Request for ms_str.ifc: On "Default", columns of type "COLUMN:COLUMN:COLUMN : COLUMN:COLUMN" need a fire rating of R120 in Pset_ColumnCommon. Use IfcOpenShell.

First a look at what the model holds.

```python
import ifcopenshell
import ifcopenshell.util.element

model = ifcopenshell.open("ms_str.ifc")
print(model.schema)
storey = next(s for s in model.by_type("IfcBuildingStorey") if s.Name == "Default")
columns = [e for e in ifcopenshell.util.element.get_decomposition(storey) if e.is_a("IfcColumn")]
seen = {}
for e in columns:
    element_type = ifcopenshell.util.element.get_type(e)
    key = (element_type.Name if element_type != e and element_type else None, ifcopenshell.util.element.get_pset(e, "Pset_ColumnCommon", "FireRating"))
    seen[key] = seen.get(key, 0) + 1
for (name, value), count in sorted(seen.items(), key=str):
    print(count, "x", name, "|", value)
```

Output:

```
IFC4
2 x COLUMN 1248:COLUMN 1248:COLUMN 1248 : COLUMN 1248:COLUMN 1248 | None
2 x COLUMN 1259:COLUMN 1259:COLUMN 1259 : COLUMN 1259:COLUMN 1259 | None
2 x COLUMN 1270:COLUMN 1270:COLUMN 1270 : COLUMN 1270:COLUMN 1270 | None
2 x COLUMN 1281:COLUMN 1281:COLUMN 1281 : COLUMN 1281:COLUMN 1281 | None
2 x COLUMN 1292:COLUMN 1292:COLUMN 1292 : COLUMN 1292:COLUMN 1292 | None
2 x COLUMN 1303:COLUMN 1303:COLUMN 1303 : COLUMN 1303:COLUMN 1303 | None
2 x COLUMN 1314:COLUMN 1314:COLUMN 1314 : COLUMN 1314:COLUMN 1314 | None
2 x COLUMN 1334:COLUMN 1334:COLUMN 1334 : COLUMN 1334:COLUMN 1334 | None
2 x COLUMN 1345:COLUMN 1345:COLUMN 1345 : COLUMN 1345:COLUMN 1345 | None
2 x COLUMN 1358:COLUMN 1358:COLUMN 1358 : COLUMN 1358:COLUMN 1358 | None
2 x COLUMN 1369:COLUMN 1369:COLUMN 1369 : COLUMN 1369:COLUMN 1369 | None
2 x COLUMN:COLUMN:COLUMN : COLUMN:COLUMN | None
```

```python
import ifcopenshell
import ifcopenshell.api.pset
import ifcopenshell.util.element

model = ifcopenshell.open("ms_str.ifc")

storey = next(s for s in model.by_type("IfcBuildingStorey") if s.Name == "Default")
columns = [e for e in ifcopenshell.util.element.get_decomposition(storey) if e.is_a("IfcColumn")]

count = 0
for e in columns:
    element_type = ifcopenshell.util.element.get_type(e)
    if element_type in (None, e) or element_type.Name != "COLUMN:COLUMN:COLUMN : COLUMN:COLUMN":
        continue
    # add_pset returns the element's existing set when there is one.
    pset = ifcopenshell.api.pset.add_pset(model, product=e, name="Pset_ColumnCommon")
    ifcopenshell.api.pset.edit_pset(model, pset=pset, properties={"FireRating": "R120"})
    count += 1

print(count, "columns updated")

model.write("ms_str_edited.ifc")
```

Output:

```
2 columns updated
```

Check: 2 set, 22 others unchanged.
